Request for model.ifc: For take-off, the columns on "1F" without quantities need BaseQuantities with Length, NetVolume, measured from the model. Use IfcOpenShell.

First a look at what the model holds.

```python
import ifcopenshell
import ifcopenshell.util.element
import ifcopenshell.util.unit

model = ifcopenshell.open("model.ifc")
print(model.schema)
for unit_type in ("LENGTHUNIT", "AREAUNIT", "VOLUMEUNIT"):
    print(unit_type, ifcopenshell.util.unit.calculate_unit_scale(model, unit_type))
storey = next(s for s in model.by_type("IfcBuildingStorey") if s.Name == "1F")
columns = [e for e in ifcopenshell.util.element.get_decomposition(storey) if e.is_a("IfcColumn")]
for e in sorted(columns, key=lambda e: e.id()):
    print(e.id(), e.is_a(), e.Name, list(ifcopenshell.util.element.get_psets(e, qtos_only=True)), sep=" | ")
```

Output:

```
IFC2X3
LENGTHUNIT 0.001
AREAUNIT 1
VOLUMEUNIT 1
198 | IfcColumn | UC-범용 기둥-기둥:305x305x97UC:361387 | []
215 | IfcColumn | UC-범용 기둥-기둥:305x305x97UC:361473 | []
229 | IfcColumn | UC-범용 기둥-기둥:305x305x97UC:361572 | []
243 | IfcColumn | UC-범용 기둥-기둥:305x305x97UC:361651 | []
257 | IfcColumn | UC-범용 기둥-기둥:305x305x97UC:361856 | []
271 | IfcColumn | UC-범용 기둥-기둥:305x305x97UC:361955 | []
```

```python
import ifcopenshell
import ifcopenshell.api.pset
import ifcopenshell.geom
import ifcopenshell.util.element
import ifcopenshell.util.shape
import ifcopenshell.util.unit

model = ifcopenshell.open("model.ifc")
unit_scale = ifcopenshell.util.unit.calculate_unit_scale(model)
volume_scale = ifcopenshell.util.unit.calculate_unit_scale(model, "VOLUMEUNIT")
settings = ifcopenshell.geom.settings()

storey = next(s for s in model.by_type("IfcBuildingStorey") if s.Name == "1F")
columns = [e for e in ifcopenshell.util.element.get_decomposition(storey) if e.is_a("IfcColumn")]

for e in sorted(columns, key=lambda e: e.id()):
    if ifcopenshell.util.element.get_psets(e, qtos_only=True, should_inherit=False):
        continue
    # Geometry comes back in metres, in the element's own axes.
    shape = ifcopenshell.geom.create_shape(settings, e)
    values = {
        "Length": ifcopenshell.util.shape.get_z(shape.geometry) / unit_scale,
        "NetVolume": ifcopenshell.util.shape.get_volume(shape.geometry) / volume_scale,
    }
    qto = ifcopenshell.api.pset.add_qto(model, product=e, name="BaseQuantities")
    ifcopenshell.api.pset.edit_qto(model, qto=qto, properties=values)
    print(e.id(), {k: round(v, 3) for k, v in values.items()})

model.write("model-out.ifc")
```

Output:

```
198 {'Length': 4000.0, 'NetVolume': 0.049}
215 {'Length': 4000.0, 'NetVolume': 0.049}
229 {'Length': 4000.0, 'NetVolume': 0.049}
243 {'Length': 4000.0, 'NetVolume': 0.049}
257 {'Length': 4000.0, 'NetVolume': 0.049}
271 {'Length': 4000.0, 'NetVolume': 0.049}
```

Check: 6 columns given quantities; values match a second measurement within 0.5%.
